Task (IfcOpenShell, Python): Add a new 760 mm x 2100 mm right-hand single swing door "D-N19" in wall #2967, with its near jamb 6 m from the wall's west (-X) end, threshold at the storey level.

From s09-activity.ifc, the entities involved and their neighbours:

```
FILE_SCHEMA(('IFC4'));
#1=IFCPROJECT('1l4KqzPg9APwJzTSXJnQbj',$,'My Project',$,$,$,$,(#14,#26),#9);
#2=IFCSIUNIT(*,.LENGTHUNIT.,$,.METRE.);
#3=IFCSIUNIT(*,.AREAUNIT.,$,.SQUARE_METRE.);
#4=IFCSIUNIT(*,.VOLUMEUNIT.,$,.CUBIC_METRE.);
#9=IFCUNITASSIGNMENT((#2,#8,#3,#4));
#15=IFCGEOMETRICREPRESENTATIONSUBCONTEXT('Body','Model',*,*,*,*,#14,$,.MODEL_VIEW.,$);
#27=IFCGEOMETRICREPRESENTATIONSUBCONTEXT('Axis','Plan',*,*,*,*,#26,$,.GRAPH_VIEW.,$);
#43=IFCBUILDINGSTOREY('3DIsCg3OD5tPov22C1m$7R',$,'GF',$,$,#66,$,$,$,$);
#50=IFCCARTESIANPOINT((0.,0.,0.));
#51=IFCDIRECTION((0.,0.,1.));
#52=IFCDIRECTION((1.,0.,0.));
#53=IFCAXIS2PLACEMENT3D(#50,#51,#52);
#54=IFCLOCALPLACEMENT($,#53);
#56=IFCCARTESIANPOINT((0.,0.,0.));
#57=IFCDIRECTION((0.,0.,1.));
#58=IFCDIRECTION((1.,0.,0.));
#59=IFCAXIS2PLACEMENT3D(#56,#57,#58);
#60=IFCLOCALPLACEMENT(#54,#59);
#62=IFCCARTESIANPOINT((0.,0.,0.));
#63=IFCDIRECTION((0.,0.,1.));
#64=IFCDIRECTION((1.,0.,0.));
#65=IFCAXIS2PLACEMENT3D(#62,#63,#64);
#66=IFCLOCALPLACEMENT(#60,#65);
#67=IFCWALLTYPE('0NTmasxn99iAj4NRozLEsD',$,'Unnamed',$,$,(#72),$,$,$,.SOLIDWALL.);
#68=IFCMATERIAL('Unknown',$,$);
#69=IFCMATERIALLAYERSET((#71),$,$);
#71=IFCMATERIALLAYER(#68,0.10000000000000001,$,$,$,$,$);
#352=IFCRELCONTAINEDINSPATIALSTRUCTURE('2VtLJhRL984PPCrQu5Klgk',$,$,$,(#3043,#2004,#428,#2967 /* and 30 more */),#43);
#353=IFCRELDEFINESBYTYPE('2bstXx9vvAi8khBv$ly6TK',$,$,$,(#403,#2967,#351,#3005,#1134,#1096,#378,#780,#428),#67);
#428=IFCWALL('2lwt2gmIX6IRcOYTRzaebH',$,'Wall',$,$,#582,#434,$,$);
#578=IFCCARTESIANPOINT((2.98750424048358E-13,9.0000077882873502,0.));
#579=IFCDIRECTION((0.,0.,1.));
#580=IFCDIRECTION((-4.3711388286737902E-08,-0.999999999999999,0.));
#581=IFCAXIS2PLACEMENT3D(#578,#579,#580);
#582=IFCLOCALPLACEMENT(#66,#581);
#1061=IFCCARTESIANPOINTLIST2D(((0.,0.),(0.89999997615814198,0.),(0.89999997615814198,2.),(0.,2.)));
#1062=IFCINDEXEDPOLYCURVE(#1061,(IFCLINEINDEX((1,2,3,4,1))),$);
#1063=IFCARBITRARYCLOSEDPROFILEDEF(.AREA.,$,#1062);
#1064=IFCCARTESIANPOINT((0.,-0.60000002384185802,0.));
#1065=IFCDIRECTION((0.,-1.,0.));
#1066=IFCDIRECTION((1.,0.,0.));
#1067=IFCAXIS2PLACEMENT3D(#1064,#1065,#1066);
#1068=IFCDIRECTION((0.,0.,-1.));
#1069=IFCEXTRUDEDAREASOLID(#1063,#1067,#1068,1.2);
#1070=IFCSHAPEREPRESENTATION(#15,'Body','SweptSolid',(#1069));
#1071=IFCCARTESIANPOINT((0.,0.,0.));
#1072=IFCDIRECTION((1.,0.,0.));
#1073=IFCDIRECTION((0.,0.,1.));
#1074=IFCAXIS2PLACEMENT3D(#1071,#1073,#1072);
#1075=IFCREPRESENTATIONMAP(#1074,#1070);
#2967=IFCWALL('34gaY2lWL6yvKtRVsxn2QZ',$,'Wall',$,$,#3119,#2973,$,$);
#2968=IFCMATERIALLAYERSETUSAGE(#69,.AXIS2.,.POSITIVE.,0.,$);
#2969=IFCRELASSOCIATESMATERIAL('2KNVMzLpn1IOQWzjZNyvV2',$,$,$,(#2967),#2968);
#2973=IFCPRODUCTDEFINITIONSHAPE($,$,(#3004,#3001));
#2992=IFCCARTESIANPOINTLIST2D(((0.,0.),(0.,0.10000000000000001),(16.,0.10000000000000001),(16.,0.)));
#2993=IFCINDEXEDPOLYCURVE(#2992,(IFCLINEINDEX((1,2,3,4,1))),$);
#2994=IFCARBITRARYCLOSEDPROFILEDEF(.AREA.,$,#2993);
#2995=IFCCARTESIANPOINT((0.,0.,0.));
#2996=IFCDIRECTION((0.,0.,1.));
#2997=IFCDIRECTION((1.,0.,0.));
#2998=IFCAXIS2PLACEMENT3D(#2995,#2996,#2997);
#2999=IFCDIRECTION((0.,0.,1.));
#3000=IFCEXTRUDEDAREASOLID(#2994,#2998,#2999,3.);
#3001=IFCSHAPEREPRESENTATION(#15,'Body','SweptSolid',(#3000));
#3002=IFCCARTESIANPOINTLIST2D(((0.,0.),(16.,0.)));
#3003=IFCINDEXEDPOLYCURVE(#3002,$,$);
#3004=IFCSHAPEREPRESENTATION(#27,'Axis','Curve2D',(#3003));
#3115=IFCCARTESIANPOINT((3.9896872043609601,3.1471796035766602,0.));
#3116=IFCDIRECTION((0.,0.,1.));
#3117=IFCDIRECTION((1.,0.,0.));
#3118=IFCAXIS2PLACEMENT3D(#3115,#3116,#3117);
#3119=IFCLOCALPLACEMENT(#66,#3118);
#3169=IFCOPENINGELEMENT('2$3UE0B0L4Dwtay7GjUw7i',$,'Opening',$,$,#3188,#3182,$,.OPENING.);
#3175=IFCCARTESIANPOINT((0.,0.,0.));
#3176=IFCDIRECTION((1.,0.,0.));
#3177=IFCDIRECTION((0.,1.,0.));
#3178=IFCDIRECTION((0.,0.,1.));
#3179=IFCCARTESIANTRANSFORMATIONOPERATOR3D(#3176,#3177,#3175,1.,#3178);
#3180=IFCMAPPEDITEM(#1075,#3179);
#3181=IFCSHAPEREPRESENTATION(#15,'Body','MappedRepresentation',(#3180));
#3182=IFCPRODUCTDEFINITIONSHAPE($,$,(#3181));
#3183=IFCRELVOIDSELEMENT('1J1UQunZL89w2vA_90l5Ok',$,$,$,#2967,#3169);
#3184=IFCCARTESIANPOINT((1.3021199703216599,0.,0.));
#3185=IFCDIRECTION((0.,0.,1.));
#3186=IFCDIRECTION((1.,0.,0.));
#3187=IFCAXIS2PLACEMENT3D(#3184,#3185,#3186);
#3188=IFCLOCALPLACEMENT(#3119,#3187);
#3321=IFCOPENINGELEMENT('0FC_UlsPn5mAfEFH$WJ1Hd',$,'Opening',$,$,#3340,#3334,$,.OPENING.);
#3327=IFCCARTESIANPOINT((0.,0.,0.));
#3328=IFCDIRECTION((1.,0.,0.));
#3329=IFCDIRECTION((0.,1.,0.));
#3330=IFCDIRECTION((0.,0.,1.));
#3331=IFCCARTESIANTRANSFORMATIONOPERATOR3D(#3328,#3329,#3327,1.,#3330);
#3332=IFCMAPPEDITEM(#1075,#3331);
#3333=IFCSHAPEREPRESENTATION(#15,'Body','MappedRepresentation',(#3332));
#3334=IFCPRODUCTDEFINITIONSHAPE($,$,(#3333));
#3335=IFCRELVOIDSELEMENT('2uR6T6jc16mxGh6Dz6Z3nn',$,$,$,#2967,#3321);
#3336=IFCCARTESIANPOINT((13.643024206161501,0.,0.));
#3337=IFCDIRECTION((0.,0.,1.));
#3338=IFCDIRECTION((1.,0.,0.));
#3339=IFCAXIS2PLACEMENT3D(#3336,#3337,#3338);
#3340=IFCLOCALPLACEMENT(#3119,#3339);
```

```python
import numpy as np
import ifcopenshell
import ifcopenshell.api.feature
import ifcopenshell.api.geometry
import ifcopenshell.api.root
import ifcopenshell.api.spatial
import ifcopenshell.geom
import ifcopenshell.util.element
import ifcopenshell.util.placement
import ifcopenshell.util.representation
import ifcopenshell.util.shape
import ifcopenshell.util.unit

model = ifcopenshell.open("s09-activity.ifc")
unit_scale = ifcopenshell.util.unit.calculate_unit_scale(model)
settings = ifcopenshell.geom.settings()


def volume(element):
    """Net volume in cubic metres, openings subtracted."""
    shape = ifcopenshell.geom.create_shape(settings, element)
    return ifcopenshell.util.shape.get_volume(shape.geometry)


wall = model.by_guid("34gaY2lWL6yvKtRVsxn2QZ")
storey = ifcopenshell.util.element.get_container(wall, ifc_class="IfcBuildingStorey")
context = ifcopenshell.util.representation.get_context(model, "Model", "Body", "MODEL_VIEW")
before = volume(wall)

width, height, from_end, sill = 0.76, 2.1, 6, 0.0  # metres

# The wall runs along its own X axis, and the end named is its -X end.
wall_shape = ifcopenshell.geom.create_shape(settings, wall)
x, y, z = ifcopenshell.util.shape.get_vertices(wall_shape.geometry).T
start = x.min() + from_end
face, thickness = float(y.min()), float(y.max() - y.min())
wall_matrix = ifcopenshell.util.placement.get_local_placement(wall.ObjectPlacement)
level = ifcopenshell.util.placement.get_local_placement(storey.ObjectPlacement)[2, 3]


def in_wall(x, y):
    """Placement at x, y metres in the wall's axes, at sill height."""
    matrix = wall_matrix.copy()
    matrix[:, 3] = wall_matrix @ np.array([x / unit_scale, y / unit_scale, 0.0, 1.0])
    matrix[2, 3] = level + sill / unit_scale
    return matrix


# Opening: a box that overshoots both wall faces by 50 mm.
opening = ifcopenshell.api.root.create_entity(model, ifc_class="IfcOpeningElement", predefined_type="OPENING")
box = ifcopenshell.api.geometry.add_wall_representation(
    model, context=context, length=width, height=height, thickness=thickness + 0.1
)
ifcopenshell.api.geometry.assign_representation(model, product=opening, representation=box)
ifcopenshell.api.geometry.edit_object_placement(model, product=opening, matrix=in_wall(start, face - 0.05), is_si=False)
ifcopenshell.api.feature.add_feature(model, feature=opening, element=wall)

door = ifcopenshell.api.root.create_entity(model, ifc_class="IfcDoor", name="D-N19", predefined_type="DOOR")
door.OverallWidth, door.OverallHeight = width / unit_scale, height / unit_scale
door.OperationType = "SINGLE_SWING_RIGHT"
body = ifcopenshell.api.geometry.add_door_representation(
    model,
    context=context,
    overall_width=door.OverallWidth,
    overall_height=door.OverallHeight,
    operation_type="SINGLE_SWING_RIGHT",
    lining_properties={"LiningDepth": thickness / unit_scale, "ThresholdDepth": thickness / unit_scale},
)
ifcopenshell.api.geometry.assign_representation(model, product=door, representation=body)
ifcopenshell.api.spatial.assign_container(model, products=[door], relating_structure=storey)
ifcopenshell.api.feature.add_filling(model, opening=opening, element=door)

# The lining spans the wall, so the door starts at the wall face.
ifcopenshell.api.geometry.edit_object_placement(model, product=door, matrix=in_wall(start, face), is_si=False)

after = volume(wall)

print(f"wall volume {before:.3f} -> {after:.3f} m3")

model.write("s09-activity_edited.ifc")
```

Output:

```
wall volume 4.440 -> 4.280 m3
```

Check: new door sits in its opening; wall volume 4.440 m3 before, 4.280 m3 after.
